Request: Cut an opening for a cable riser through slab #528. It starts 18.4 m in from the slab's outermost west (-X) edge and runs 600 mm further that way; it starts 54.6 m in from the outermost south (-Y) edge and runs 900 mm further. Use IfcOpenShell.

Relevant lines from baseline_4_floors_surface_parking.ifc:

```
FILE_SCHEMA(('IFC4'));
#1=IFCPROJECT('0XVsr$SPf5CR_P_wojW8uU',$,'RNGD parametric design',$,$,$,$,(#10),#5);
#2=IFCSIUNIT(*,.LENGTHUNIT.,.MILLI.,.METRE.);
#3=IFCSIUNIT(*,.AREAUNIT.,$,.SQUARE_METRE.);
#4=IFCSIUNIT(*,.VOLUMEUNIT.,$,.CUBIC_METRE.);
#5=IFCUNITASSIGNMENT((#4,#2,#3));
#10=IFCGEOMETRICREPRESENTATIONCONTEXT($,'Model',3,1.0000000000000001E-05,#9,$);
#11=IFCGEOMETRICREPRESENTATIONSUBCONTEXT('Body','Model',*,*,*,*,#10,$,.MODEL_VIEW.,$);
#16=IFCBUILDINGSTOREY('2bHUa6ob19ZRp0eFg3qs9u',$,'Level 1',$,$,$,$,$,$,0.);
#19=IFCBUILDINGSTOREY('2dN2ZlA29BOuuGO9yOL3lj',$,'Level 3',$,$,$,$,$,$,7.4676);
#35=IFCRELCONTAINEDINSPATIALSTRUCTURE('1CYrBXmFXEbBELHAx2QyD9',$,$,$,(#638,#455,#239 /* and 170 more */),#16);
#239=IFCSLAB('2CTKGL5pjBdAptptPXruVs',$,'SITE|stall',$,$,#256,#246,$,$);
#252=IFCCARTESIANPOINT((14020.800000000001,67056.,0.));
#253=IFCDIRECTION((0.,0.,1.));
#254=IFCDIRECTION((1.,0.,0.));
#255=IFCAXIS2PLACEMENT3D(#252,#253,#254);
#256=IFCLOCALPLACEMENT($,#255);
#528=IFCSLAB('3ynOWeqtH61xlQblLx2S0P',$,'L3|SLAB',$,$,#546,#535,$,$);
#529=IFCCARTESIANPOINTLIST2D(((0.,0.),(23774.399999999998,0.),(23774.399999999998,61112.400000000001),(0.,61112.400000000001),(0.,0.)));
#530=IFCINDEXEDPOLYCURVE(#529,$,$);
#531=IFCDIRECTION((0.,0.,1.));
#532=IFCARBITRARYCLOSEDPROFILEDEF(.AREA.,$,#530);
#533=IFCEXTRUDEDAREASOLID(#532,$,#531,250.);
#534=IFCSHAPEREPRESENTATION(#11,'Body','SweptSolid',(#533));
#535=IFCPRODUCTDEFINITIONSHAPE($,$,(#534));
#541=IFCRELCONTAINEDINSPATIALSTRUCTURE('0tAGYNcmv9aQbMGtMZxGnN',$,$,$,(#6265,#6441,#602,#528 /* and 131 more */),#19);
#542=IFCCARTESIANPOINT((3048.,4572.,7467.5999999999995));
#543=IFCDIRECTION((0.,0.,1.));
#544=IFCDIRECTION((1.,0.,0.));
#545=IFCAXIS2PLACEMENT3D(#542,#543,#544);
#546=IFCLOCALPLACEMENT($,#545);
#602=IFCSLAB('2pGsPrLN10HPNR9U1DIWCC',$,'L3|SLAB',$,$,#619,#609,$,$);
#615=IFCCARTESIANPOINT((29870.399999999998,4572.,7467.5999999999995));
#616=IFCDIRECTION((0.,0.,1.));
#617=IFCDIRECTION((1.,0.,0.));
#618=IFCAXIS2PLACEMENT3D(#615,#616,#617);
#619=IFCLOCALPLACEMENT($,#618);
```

```python
import numpy as np
import ifcopenshell
import ifcopenshell.api.feature
import ifcopenshell.api.geometry
import ifcopenshell.api.root
import ifcopenshell.geom
import ifcopenshell.util.placement
import ifcopenshell.util.representation
import ifcopenshell.util.shape
import ifcopenshell.util.unit

model = ifcopenshell.open("baseline_4_floors_surface_parking.ifc")
unit_scale = ifcopenshell.util.unit.calculate_unit_scale(model)
settings = ifcopenshell.geom.settings()


def volume(element):
    """Net volume in cubic metres, openings subtracted."""
    shape = ifcopenshell.geom.create_shape(settings, element)
    return ifcopenshell.util.shape.get_volume(shape.geometry)


slab = model.by_guid("3ynOWeqtH61xlQblLx2S0P")
before = volume(slab)

# Extent in the slab's own axes, in metres. The edges named are its -X and -Y sides.
slab_shape = ifcopenshell.geom.create_shape(settings, slab)
vertices = ifcopenshell.util.shape.get_vertices(slab_shape.geometry)
x_min, y_min, bottom = vertices.min(axis=0)
top = vertices[:, 2].max()

opening = ifcopenshell.api.root.create_entity(model, ifc_class="IfcOpeningElement", name="Cable riser opening", predefined_type="OPENING")
context = ifcopenshell.util.representation.get_context(model, "Model", "Body", "MODEL_VIEW")
width, depth = 0.6, 0.9
outline = [(0.0, 0.0), (width, 0.0), (width, depth), (0.0, depth), (0.0, 0.0)]
# Overshoot both faces by 50 mm so the cut is clean.
shape = ifcopenshell.api.geometry.add_slab_representation(
    model, context=context, depth=top - bottom + 0.1, polyline=outline
)
ifcopenshell.api.geometry.assign_representation(model, product=opening, representation=shape)

matrix = ifcopenshell.util.placement.get_local_placement(slab.ObjectPlacement)
matrix[:, 3] = matrix @ np.append(np.array([x_min + 18.4, y_min + 54.6, bottom - 0.05]) / unit_scale, 1.0)
ifcopenshell.api.geometry.edit_object_placement(model, product=opening, matrix=matrix, is_si=False)
ifcopenshell.api.feature.add_feature(model, feature=opening, element=slab)

after = volume(slab)

print(f"slab volume {before:.3f} -> {after:.3f} m3")

model.write("baseline_4_floors_surface_parking-out.ifc")
```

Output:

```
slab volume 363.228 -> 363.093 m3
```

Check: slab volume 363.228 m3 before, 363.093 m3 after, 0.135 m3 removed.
